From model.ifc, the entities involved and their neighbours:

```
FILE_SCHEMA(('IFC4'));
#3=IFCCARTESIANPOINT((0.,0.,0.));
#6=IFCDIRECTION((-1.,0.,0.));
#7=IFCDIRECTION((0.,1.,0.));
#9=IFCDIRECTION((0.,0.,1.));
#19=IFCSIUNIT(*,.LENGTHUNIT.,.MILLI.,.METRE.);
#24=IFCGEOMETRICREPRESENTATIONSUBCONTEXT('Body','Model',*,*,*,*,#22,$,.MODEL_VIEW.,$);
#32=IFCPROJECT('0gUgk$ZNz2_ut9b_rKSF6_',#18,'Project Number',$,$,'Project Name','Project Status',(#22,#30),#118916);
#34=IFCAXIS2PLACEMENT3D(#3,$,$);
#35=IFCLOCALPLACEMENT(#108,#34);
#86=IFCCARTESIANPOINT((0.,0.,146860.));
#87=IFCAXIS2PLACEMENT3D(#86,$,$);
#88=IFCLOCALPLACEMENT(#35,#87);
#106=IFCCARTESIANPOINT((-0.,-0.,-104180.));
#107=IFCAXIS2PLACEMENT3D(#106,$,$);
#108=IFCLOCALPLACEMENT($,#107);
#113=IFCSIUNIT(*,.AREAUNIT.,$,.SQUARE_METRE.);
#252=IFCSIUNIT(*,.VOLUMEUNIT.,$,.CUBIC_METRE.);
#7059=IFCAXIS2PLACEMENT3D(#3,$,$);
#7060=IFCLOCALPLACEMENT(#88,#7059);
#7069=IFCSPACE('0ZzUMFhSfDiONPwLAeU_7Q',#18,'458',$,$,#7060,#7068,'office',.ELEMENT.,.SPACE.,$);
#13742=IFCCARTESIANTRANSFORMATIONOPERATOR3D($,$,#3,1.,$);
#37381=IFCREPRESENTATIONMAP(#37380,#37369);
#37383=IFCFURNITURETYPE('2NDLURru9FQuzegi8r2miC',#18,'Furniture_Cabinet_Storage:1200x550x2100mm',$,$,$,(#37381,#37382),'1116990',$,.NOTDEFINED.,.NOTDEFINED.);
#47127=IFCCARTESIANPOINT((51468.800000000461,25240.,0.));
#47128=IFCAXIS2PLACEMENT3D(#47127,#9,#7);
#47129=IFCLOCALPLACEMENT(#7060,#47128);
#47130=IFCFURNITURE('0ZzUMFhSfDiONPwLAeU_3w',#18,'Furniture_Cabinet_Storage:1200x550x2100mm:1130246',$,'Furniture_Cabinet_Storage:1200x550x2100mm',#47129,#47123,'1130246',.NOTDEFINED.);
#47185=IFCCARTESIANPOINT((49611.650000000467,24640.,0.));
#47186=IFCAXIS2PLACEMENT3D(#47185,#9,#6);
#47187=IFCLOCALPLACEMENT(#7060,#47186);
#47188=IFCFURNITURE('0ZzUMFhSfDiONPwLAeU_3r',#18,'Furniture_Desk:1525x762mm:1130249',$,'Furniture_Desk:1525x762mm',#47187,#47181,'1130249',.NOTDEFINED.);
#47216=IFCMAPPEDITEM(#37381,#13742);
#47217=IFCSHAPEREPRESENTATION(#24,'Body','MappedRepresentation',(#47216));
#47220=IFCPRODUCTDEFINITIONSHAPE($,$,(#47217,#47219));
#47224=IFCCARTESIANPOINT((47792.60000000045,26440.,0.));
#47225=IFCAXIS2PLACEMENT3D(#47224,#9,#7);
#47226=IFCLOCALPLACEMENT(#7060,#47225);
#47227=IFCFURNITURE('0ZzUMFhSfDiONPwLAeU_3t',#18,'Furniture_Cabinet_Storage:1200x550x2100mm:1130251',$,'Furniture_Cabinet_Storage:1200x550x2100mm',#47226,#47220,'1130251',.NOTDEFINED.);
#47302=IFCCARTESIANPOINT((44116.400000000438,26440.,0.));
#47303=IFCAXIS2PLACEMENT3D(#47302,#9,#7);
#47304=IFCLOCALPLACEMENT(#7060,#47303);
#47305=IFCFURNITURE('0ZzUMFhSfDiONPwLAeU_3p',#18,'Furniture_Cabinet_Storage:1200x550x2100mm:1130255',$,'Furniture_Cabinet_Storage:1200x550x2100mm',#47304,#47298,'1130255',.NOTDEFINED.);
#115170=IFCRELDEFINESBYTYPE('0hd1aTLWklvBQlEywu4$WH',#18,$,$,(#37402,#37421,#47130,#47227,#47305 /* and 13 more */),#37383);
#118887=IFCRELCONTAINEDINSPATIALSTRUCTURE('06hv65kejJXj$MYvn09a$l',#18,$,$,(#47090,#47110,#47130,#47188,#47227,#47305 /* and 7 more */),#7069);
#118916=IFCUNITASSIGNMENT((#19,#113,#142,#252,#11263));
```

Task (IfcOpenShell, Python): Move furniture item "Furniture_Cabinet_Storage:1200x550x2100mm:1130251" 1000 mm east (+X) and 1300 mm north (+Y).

```python
import ifcopenshell
import ifcopenshell.api.geometry
import ifcopenshell.util.placement
import ifcopenshell.util.unit

model = ifcopenshell.open("model.ifc")
unit_scale = ifcopenshell.util.unit.calculate_unit_scale(model)

item = model.by_guid("0ZzUMFhSfDiONPwLAeU_3t")
matrix = ifcopenshell.util.placement.get_local_placement(item.ObjectPlacement)
matrix[0, 3] += 1 / unit_scale
matrix[1, 3] += 1.3 / unit_scale
ifcopenshell.api.geometry.edit_object_placement(model, product=item, matrix=matrix, is_si=False)

print(ifcopenshell.util.placement.get_local_placement(item.ObjectPlacement).round(3) + 0.0)

model.write("model_edited.ifc")
```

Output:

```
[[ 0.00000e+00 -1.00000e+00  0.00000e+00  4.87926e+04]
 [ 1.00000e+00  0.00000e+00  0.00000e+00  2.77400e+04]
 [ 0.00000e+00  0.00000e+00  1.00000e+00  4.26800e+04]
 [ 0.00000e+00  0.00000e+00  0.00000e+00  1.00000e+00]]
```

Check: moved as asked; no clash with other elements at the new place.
